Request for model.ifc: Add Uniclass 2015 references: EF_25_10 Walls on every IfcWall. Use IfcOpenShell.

First a look at what the model holds.

```python
import ifcopenshell

model = ifcopenshell.open("model.ifc")
print(model.schema)
print("classifications:", [c.Name for c in model.by_type("IfcClassification")])
for ifc_class in ("IfcDoor", "IfcRoof", "IfcStair", "IfcWall", "IfcWindow"):
    print(ifc_class, len(model.by_type(ifc_class)))
```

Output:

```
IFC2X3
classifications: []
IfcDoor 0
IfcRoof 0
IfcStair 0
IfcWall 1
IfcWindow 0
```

```python
import ifcopenshell
import ifcopenshell.api.classification

model = ifcopenshell.open("model.ifc")

# IFC2X3 requires Source and Edition and has no link from the project to the system.
system = model.create_entity("IfcClassification", Source="NBS", Edition="2015", Name="Uniclass 2015")

codes = {
    "IfcWall": ("EF_25_10", "Walls"),
}
for ifc_class, (code, name) in codes.items():
    products = model.by_type(ifc_class)
    ifcopenshell.api.classification.add_reference(
        model, products=products, classification=system, identification=code, name=name
    )
    print(code, len(products))

model.write("model_v2.ifc")
```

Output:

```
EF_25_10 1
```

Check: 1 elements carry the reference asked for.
